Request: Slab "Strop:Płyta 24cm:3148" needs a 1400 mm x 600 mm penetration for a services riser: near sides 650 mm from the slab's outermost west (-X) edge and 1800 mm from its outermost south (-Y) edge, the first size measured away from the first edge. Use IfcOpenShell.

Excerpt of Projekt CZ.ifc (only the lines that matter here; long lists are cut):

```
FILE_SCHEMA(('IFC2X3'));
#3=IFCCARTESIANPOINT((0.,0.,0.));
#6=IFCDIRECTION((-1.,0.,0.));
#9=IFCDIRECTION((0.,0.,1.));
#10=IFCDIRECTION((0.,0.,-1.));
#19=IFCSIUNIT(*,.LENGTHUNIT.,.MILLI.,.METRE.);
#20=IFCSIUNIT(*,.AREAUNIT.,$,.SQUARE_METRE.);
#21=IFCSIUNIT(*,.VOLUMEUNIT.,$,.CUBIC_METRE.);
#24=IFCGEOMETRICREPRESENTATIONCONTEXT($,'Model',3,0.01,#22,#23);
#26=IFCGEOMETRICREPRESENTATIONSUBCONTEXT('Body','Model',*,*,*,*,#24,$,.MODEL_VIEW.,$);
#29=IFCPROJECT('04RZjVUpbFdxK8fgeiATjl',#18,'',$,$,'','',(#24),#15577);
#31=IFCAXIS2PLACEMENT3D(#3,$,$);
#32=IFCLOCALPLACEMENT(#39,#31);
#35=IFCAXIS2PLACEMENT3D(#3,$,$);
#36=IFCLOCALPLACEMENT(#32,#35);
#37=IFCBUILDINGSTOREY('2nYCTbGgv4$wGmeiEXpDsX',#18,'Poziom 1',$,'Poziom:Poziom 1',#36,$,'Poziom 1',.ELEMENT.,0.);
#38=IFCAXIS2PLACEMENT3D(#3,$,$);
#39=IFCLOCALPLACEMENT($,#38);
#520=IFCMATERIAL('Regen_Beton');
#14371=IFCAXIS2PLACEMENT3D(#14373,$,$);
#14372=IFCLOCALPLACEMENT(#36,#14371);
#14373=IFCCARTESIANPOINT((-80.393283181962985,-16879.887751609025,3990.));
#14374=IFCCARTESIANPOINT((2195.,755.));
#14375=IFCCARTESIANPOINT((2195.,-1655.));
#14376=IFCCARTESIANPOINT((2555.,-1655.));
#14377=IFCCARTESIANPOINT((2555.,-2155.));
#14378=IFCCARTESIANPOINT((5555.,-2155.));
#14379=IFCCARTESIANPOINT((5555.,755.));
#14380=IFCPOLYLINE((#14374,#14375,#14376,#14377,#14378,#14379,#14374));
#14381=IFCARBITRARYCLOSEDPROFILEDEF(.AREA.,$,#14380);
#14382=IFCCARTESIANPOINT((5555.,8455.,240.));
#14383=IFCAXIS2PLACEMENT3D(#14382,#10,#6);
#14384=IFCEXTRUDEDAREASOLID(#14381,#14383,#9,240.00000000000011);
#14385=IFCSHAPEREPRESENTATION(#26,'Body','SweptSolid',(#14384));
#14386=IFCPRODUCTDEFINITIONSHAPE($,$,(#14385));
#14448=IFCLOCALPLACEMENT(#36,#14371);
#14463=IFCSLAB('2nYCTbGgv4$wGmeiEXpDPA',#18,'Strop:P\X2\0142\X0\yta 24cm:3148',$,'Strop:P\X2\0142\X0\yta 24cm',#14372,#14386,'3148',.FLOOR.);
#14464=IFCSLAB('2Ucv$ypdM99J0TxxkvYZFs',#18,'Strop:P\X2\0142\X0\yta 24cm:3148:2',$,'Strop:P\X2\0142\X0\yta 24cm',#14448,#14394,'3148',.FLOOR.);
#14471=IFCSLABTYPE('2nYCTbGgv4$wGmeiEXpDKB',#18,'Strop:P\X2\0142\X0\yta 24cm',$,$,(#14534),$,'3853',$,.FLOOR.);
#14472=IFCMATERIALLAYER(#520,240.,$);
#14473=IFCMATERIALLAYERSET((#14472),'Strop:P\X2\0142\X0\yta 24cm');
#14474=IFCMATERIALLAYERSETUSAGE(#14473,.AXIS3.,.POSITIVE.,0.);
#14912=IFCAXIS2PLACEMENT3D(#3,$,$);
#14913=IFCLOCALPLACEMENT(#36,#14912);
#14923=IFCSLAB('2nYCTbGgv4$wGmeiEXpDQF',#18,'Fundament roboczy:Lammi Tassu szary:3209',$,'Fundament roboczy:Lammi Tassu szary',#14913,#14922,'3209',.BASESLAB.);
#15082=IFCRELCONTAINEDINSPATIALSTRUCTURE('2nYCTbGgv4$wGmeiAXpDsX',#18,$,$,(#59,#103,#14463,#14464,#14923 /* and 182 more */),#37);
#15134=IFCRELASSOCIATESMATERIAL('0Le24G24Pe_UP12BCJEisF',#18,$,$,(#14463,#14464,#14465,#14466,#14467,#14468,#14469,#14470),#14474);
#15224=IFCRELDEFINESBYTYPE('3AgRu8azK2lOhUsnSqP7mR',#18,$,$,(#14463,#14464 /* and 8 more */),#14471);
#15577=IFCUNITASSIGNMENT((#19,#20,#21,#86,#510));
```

```python
import numpy as np
import ifcopenshell
import ifcopenshell.api.feature
import ifcopenshell.api.geometry
import ifcopenshell.api.root
import ifcopenshell.geom
import ifcopenshell.util.placement
import ifcopenshell.util.representation
import ifcopenshell.util.shape
import ifcopenshell.util.unit

model = ifcopenshell.open("Projekt CZ.ifc")
unit_scale = ifcopenshell.util.unit.calculate_unit_scale(model)
settings = ifcopenshell.geom.settings()


def volume(element):
    """Net volume in cubic metres, openings subtracted."""
    shape = ifcopenshell.geom.create_shape(settings, element)
    return ifcopenshell.util.shape.get_volume(shape.geometry)


slab = model.by_guid("2nYCTbGgv4$wGmeiEXpDPA")
before = volume(slab)

# Extent in the slab's own axes, in metres. The edges named are its -X and -Y sides.
slab_shape = ifcopenshell.geom.create_shape(settings, slab)
vertices = ifcopenshell.util.shape.get_vertices(slab_shape.geometry)
x_min, y_min, bottom = vertices.min(axis=0)
top = vertices[:, 2].max()

opening = ifcopenshell.api.root.create_entity(model, ifc_class="IfcOpeningElement", name="Services riser opening")
context = ifcopenshell.util.representation.get_context(model, "Model", "Body", "MODEL_VIEW")
width, depth = 1.4, 0.6
outline = [(0.0, 0.0), (width, 0.0), (width, depth), (0.0, depth), (0.0, 0.0)]
# Overshoot both faces by 50 mm so the cut is clean.
shape = ifcopenshell.api.geometry.add_slab_representation(
    model, context=context, depth=top - bottom + 0.1, polyline=outline
)
ifcopenshell.api.geometry.assign_representation(model, product=opening, representation=shape)

matrix = ifcopenshell.util.placement.get_local_placement(slab.ObjectPlacement)
matrix[:, 3] = matrix @ np.append(np.array([x_min + 0.65, y_min + 1.8, bottom - 0.05]) / unit_scale, 1.0)
ifcopenshell.api.geometry.edit_object_placement(model, product=opening, matrix=matrix, is_si=False)
ifcopenshell.api.feature.add_feature(model, feature=opening, element=slab)

after = volume(slab)

print(f"slab volume {before:.3f} -> {after:.3f} m3")

model.write("Projekt CZ-out.ifc")
```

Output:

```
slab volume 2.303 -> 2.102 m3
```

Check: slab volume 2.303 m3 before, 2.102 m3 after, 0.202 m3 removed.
